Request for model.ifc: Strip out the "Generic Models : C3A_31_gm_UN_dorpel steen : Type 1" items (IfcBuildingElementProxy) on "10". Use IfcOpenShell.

First a look at what the model holds.

```python
import ifcopenshell
import ifcopenshell.util.element

model = ifcopenshell.open("model.ifc")
print(model.schema)
storey = next(s for s in model.by_type("IfcBuildingStorey") if s.Name == "10")
proxies = [e for e in ifcopenshell.util.element.get_decomposition(storey) if e.is_a("IfcBuildingElementProxy")]
seen = {}
for e in proxies:
    element_type = ifcopenshell.util.element.get_type(e)
    name = element_type.Name if element_type not in (None, e) else None
    seen[name] = seen.get(name, 0) + 1
for name, count in sorted(seen.items(), key=str):
    print(count, "x", name)
```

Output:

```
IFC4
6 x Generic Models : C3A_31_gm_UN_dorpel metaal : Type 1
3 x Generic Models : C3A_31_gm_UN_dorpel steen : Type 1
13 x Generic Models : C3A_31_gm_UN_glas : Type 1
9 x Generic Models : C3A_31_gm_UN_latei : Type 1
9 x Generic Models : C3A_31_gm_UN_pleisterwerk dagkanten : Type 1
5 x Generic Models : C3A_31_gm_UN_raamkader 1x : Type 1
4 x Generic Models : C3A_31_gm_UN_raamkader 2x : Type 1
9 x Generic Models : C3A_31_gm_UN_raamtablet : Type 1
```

```python
import ifcopenshell
import ifcopenshell.api.root
import ifcopenshell.util.element

model = ifcopenshell.open("model.ifc")

storey = next(s for s in model.by_type("IfcBuildingStorey") if s.Name == "10")
proxies = [e for e in ifcopenshell.util.element.get_decomposition(storey) if e.is_a("IfcBuildingElementProxy")]
targets = [e for e in proxies if (t := ifcopenshell.util.element.get_type(e)) not in (None, e) and t.Name == "Generic Models : C3A_31_gm_UN_dorpel steen : Type 1"]

for e in targets:
    ifcopenshell.api.root.remove_product(model, product=e)
print(len(targets), "removed")

model.write("model_edited.ifc")
```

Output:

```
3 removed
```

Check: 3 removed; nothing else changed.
